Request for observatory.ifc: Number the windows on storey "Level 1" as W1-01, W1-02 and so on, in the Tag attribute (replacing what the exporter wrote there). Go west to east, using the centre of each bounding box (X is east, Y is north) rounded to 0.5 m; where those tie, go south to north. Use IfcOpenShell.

First a look at what the model holds.

```python
import ifcopenshell
import ifcopenshell.util.element
import ifcopenshell.util.placement

model = ifcopenshell.open("observatory.ifc")
print(model.schema)
storey = next(s for s in model.by_type("IfcBuildingStorey") if s.Name == "Level 1")
windows = [e for e in ifcopenshell.util.element.get_decomposition(storey) if e.is_a("IfcWindow")]
for e in sorted(windows, key=lambda e: e.id()):
    origin = ifcopenshell.util.placement.get_local_placement(e.ObjectPlacement)[:3, 3]
    print(e.id(), e.Tag, e.Name, origin.round(2) + 0.0, sep=" | ")
```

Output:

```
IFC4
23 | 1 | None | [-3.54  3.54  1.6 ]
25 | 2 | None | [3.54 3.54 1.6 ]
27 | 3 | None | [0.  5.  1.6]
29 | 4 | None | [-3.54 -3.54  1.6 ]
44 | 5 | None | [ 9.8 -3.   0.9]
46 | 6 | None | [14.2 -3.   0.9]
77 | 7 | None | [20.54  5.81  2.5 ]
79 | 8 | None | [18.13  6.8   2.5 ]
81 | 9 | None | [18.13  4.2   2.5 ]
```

```python
import ifcopenshell
import ifcopenshell.geom
import ifcopenshell.util.element
import ifcopenshell.util.shape

model = ifcopenshell.open("observatory.ifc")
settings = ifcopenshell.geom.settings()
settings.set("use-world-coords", True)


def centre(element):
    shape = ifcopenshell.geom.create_shape(settings, element)
    return ifcopenshell.util.shape.get_bbox_centroid(shape.geometry)


storey = next(s for s in model.by_type("IfcBuildingStorey") if s.Name == "Level 1")
windows = [e for e in ifcopenshell.util.element.get_decomposition(storey) if e.is_a("IfcWindow")]

# Insertion points can sit at a corner or the storey origin, so sort by the geometry (in metres).
centres = {e: centre(e) for e in windows}
windows.sort(key=lambda e: (round(centres[e][0] / 0.5), centres[e][1]))

for i, e in enumerate(windows, start=1):
    number = f"W1-{i:02d}"
    e.Tag = number
    print(e.id(), number)

model.write("observatory-out.ifc")
```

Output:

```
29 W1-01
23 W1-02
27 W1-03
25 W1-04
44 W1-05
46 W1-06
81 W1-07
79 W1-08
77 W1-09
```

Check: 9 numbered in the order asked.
